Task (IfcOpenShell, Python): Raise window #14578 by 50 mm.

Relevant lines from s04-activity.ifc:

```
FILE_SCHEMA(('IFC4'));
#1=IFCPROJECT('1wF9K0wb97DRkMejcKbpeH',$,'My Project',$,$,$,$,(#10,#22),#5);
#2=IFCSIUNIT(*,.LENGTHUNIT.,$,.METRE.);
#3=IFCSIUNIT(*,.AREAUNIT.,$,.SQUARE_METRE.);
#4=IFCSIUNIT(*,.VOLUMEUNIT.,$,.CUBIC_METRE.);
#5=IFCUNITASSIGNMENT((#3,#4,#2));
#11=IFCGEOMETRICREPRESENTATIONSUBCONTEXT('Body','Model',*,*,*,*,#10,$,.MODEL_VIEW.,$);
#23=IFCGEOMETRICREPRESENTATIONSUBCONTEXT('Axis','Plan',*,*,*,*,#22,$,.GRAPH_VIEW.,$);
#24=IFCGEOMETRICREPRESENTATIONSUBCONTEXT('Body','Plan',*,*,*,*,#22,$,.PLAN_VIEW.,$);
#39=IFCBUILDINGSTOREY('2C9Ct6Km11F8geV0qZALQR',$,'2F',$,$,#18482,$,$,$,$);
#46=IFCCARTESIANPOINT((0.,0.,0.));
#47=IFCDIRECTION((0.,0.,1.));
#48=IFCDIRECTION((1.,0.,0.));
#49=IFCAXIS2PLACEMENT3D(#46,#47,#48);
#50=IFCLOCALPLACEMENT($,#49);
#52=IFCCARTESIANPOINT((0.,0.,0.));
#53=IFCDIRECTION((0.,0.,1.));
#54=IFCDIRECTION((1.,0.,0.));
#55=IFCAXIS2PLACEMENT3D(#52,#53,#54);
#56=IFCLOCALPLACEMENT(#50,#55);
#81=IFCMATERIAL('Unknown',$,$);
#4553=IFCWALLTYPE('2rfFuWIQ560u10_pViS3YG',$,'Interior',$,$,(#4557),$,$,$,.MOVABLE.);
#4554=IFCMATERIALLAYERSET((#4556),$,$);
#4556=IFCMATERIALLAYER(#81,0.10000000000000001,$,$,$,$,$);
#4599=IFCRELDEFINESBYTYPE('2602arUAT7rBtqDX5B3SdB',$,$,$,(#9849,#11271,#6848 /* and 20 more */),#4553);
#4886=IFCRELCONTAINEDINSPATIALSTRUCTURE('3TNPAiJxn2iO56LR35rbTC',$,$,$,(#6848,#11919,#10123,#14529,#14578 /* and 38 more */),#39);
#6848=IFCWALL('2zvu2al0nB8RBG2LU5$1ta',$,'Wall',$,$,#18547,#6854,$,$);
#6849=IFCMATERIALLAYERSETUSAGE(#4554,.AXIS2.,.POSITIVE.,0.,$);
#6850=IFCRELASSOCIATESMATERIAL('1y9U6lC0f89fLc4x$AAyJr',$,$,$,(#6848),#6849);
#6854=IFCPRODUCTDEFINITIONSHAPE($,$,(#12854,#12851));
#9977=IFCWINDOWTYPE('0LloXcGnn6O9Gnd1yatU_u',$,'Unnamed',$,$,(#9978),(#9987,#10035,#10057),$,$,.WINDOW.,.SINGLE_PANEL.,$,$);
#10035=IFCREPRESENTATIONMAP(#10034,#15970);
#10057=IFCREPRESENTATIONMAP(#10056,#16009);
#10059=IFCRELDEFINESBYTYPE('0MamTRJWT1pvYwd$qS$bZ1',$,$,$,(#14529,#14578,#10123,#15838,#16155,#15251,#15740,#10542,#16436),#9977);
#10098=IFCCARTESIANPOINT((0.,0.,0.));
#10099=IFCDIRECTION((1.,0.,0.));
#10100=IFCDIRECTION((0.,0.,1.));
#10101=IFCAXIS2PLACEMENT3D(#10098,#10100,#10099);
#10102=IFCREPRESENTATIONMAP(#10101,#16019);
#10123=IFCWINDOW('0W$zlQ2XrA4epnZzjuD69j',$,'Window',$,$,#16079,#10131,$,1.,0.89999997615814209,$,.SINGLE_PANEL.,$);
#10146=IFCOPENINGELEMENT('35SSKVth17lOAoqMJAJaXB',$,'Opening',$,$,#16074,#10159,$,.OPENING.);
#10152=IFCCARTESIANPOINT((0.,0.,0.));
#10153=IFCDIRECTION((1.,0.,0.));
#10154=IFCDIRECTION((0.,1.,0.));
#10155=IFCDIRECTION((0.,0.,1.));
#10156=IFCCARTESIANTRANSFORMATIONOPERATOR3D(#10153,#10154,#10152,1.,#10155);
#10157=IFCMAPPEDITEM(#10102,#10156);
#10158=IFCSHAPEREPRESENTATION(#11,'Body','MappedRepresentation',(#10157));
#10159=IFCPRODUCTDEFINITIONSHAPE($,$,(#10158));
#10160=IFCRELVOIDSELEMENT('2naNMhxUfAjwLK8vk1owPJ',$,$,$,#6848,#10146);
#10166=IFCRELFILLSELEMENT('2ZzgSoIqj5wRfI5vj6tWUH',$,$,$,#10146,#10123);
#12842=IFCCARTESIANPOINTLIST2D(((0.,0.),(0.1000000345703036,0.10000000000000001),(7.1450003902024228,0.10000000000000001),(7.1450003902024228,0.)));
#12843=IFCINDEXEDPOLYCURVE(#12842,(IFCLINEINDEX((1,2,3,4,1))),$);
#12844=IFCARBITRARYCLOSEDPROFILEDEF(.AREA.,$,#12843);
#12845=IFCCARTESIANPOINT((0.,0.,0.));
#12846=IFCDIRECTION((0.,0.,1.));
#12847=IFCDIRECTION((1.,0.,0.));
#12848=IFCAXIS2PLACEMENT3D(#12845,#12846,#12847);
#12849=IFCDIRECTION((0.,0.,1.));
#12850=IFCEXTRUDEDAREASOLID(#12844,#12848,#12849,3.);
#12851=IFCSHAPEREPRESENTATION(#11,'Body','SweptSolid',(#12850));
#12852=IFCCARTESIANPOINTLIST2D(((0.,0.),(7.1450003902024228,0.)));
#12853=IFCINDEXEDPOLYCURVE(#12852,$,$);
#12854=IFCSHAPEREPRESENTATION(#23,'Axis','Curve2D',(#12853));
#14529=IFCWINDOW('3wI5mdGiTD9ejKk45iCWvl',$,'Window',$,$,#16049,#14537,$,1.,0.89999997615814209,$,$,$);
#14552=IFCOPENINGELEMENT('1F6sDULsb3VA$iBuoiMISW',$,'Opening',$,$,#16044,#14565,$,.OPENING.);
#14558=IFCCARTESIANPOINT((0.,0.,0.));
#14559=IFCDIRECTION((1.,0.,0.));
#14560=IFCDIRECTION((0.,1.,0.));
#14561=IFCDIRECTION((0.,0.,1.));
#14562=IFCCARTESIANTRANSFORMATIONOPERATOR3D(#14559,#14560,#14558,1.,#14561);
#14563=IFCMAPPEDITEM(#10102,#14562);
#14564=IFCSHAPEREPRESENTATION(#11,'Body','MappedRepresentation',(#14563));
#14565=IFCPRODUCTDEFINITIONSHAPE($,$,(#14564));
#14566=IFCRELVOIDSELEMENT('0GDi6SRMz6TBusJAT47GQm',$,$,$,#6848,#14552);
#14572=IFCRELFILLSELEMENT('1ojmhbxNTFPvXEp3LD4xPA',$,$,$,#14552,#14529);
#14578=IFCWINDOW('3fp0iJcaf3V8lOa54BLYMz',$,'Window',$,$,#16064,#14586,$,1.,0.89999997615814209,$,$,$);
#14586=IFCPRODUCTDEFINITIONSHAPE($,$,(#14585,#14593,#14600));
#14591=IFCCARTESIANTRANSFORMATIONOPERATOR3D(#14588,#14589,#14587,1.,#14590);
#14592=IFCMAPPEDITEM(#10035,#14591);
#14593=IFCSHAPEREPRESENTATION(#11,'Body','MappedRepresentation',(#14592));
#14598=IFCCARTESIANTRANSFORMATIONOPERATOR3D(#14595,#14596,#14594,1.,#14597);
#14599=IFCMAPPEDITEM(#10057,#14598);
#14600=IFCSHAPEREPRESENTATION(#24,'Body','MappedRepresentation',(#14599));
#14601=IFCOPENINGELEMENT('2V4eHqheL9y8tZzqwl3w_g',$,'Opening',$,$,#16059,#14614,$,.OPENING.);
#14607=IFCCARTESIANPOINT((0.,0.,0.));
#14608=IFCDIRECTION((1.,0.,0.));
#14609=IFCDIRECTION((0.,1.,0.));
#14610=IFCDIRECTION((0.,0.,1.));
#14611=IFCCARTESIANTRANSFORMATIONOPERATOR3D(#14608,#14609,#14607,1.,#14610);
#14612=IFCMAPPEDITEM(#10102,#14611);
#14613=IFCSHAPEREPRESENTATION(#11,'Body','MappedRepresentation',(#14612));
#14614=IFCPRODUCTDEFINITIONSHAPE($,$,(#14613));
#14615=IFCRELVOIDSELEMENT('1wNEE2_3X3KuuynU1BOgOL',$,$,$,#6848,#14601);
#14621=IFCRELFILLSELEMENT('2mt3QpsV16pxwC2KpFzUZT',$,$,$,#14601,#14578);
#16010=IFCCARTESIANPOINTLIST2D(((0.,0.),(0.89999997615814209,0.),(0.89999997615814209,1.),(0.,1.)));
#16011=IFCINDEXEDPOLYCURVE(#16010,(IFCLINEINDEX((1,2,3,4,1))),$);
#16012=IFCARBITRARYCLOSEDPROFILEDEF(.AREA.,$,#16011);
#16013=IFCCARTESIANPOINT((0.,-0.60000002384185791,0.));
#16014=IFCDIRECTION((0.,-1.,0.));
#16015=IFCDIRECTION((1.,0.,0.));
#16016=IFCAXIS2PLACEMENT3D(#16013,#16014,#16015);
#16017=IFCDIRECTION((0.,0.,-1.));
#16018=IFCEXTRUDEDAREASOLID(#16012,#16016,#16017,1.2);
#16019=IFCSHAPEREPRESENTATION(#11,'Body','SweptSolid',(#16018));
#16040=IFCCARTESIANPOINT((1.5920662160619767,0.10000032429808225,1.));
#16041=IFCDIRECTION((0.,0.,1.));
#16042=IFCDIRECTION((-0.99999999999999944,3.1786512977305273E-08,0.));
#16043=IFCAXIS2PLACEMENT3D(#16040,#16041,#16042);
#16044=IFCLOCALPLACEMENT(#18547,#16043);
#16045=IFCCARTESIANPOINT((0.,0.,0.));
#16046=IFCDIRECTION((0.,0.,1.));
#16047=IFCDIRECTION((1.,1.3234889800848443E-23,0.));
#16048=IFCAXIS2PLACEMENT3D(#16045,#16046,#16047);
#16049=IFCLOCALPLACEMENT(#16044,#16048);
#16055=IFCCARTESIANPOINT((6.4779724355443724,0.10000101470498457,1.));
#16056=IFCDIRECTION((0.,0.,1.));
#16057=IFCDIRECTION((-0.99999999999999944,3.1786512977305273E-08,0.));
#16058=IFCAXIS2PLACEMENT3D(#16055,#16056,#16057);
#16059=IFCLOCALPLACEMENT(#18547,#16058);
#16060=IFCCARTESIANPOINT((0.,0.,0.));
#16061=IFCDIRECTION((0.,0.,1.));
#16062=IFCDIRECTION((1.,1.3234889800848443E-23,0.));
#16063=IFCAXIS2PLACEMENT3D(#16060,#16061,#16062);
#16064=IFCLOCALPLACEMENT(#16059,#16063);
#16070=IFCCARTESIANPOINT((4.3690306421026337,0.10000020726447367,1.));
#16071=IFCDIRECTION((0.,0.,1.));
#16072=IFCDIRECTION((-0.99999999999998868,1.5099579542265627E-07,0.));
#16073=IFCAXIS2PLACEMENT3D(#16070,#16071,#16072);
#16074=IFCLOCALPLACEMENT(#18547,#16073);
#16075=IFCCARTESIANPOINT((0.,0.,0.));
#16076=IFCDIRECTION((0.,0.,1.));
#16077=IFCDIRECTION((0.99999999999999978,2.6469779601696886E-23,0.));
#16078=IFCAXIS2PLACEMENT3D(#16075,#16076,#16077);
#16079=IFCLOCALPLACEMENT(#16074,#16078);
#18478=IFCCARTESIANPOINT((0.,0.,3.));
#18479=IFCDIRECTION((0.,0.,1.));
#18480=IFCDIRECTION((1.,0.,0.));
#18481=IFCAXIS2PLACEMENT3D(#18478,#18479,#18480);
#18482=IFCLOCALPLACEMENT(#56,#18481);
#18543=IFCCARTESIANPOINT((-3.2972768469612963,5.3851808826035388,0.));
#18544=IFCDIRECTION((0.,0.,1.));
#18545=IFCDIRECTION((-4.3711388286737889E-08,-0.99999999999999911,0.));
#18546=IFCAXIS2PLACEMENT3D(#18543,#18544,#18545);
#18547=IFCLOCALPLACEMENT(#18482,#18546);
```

```python
import numpy as np
import ifcopenshell
import ifcopenshell.api.geometry
import ifcopenshell.util.placement
import ifcopenshell.util.unit

model = ifcopenshell.open("s04-activity.ifc")
unit_scale = ifcopenshell.util.unit.calculate_unit_scale(model)

window = model.by_guid("3fp0iJcaf3V8lOa54BLYMz")
opening = window.FillsVoids[0].RelatingOpeningElement
dz = 0.05 / unit_scale

shift = np.array([0.0, 0.0, dz])
# The window is placed relative to its opening, so it follows when the opening moves.
matrix = ifcopenshell.util.placement.get_local_placement(opening.ObjectPlacement)
matrix[:3, 3] += shift
ifcopenshell.api.geometry.edit_object_placement(
    model, product=opening, matrix=matrix, is_si=False, should_transform_children=True
)

print(f"moved by {dz * unit_scale:+.3f} m")

model.write("s04-activity_rev.ifc")
```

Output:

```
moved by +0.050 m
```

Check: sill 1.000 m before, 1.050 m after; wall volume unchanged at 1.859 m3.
